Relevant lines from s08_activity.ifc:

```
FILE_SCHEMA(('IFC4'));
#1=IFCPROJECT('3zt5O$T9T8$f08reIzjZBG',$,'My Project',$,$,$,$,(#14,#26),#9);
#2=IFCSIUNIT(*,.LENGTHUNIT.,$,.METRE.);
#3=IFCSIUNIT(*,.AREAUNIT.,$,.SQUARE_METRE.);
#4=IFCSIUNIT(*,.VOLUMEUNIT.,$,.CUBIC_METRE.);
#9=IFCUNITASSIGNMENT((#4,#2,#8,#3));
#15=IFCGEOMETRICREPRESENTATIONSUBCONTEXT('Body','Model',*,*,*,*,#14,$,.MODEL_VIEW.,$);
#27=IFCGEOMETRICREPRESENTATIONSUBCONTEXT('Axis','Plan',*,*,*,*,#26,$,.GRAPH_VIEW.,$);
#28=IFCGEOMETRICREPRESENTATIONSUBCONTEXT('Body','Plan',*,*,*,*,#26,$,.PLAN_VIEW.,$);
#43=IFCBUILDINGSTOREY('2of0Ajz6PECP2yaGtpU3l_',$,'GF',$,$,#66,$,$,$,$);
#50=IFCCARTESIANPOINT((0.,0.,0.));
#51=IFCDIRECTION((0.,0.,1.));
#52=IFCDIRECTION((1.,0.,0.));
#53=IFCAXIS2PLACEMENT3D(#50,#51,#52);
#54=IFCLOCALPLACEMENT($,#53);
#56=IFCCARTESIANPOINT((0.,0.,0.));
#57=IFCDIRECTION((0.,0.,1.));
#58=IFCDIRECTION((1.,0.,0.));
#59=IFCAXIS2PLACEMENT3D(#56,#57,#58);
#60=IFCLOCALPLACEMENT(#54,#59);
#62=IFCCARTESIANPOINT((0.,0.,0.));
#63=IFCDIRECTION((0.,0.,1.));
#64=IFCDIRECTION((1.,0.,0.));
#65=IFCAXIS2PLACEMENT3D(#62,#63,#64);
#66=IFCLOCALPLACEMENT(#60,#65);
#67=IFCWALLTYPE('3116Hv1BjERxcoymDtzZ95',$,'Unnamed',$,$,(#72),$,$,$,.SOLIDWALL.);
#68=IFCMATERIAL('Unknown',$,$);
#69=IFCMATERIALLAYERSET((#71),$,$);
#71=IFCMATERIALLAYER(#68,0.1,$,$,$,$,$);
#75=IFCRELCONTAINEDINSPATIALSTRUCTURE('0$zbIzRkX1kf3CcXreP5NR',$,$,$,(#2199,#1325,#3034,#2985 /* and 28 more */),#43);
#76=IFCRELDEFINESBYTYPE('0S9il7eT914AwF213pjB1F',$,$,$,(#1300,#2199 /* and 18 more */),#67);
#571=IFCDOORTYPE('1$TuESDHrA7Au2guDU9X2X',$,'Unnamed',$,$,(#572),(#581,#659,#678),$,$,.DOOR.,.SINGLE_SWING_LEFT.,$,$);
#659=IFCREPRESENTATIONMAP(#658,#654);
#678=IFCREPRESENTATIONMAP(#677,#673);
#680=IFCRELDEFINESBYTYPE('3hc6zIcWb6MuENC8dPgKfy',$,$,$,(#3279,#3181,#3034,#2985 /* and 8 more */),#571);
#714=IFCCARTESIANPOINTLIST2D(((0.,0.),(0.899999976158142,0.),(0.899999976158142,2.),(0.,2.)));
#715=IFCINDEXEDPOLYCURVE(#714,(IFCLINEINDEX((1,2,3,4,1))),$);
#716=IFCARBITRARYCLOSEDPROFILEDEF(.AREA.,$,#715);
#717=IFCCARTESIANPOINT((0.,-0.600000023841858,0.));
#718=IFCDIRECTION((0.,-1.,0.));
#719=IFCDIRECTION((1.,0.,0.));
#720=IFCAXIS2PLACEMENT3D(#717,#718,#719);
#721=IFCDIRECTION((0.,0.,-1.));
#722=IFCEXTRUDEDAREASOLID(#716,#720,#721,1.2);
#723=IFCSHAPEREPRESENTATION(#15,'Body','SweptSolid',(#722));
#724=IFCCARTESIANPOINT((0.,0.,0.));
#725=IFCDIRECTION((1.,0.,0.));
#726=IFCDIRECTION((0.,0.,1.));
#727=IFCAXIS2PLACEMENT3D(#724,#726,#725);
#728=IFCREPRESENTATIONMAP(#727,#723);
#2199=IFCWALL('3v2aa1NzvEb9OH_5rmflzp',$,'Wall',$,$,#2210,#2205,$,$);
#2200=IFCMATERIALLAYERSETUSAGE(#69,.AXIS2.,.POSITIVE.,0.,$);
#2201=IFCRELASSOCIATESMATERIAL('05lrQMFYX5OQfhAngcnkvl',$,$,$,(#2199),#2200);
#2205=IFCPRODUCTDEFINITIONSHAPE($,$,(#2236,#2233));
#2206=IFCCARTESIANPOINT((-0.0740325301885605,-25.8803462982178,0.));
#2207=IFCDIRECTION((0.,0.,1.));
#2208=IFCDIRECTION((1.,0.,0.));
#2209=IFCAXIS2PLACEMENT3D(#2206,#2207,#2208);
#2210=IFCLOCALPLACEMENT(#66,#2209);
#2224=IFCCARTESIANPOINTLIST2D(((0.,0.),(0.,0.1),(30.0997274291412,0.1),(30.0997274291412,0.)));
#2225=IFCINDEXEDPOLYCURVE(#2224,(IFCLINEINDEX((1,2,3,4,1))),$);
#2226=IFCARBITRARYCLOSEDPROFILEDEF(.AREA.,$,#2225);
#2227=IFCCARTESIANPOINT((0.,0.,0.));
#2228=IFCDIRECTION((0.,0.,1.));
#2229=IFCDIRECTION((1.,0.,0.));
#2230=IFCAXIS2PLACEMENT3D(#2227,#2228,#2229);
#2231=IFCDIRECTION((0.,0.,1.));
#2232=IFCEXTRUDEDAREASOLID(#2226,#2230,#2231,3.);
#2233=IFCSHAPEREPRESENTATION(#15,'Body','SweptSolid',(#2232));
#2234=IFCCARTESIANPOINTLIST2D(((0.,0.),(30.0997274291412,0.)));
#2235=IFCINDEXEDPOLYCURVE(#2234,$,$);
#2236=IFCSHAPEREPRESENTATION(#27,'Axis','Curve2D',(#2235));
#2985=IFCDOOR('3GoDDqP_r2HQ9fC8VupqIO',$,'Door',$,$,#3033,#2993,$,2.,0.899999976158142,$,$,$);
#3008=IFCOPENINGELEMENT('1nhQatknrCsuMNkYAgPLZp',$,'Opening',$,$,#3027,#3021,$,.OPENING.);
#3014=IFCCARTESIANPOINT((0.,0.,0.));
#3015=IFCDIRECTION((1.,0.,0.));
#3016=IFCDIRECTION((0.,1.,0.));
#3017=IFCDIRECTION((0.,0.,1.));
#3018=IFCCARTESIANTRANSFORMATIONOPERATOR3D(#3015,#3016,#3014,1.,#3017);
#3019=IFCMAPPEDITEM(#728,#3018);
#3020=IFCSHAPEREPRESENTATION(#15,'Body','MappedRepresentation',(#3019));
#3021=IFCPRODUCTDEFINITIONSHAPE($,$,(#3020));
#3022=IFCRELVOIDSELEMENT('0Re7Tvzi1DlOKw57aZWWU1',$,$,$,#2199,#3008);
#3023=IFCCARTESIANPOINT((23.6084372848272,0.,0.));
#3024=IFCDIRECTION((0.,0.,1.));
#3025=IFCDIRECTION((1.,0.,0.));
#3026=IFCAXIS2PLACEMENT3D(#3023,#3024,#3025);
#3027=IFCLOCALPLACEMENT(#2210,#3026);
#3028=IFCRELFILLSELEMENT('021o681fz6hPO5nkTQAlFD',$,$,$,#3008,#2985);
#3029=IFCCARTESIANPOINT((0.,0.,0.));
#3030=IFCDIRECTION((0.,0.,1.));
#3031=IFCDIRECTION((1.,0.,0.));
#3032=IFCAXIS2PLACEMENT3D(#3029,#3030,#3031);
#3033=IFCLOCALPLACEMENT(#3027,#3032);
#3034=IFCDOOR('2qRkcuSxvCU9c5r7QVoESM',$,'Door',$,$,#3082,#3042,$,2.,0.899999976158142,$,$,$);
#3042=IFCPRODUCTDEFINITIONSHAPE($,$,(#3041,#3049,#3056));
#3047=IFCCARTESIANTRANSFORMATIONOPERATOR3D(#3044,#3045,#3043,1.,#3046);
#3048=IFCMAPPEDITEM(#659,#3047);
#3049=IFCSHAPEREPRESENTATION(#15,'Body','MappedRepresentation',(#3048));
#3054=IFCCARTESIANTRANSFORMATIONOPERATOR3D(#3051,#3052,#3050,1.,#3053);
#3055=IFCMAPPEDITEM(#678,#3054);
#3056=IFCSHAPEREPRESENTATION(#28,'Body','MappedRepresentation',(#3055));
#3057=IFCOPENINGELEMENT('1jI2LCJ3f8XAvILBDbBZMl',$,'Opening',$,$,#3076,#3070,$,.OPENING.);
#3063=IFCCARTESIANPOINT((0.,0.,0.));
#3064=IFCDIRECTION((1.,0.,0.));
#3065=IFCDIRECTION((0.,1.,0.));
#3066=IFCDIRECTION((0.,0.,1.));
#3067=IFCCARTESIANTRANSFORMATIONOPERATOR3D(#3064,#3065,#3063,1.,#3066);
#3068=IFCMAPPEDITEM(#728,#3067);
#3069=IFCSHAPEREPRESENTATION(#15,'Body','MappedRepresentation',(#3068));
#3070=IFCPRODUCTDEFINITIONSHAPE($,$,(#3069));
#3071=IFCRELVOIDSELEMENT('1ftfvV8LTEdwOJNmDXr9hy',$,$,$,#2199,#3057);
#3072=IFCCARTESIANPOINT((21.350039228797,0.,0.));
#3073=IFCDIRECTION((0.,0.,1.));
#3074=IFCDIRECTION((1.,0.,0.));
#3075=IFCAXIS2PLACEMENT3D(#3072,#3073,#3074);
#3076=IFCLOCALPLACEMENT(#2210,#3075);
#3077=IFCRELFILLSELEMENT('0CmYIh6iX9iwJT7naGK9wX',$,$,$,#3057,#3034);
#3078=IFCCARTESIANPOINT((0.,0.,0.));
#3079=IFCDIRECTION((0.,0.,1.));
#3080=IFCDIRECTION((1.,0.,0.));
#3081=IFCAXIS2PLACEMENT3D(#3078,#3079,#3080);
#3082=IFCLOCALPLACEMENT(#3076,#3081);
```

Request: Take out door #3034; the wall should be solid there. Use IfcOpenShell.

```python
import ifcopenshell
import ifcopenshell.api.feature
import ifcopenshell.api.root
import ifcopenshell.geom
import ifcopenshell.util.shape

model = ifcopenshell.open("s08_activity.ifc")
settings = ifcopenshell.geom.settings()


def volume(element):
    """Net volume in cubic metres, openings subtracted."""
    shape = ifcopenshell.geom.create_shape(settings, element)
    return ifcopenshell.util.shape.get_volume(shape.geometry)


door = model.by_guid("2qRkcuSxvCU9c5r7QVoESM")
opening = door.FillsVoids[0].RelatingOpeningElement
wall = opening.VoidsElements[0].RelatingBuildingElement
before = volume(wall)

ifcopenshell.api.root.remove_product(model, product=door)
ifcopenshell.api.feature.remove_feature(model, feature=opening)

after = volume(wall)

print(f"wall volume {before:.3f} -> {after:.3f} m3")

model.write("s08_activity-out.ifc")
```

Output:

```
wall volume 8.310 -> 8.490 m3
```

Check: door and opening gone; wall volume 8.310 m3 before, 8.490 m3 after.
